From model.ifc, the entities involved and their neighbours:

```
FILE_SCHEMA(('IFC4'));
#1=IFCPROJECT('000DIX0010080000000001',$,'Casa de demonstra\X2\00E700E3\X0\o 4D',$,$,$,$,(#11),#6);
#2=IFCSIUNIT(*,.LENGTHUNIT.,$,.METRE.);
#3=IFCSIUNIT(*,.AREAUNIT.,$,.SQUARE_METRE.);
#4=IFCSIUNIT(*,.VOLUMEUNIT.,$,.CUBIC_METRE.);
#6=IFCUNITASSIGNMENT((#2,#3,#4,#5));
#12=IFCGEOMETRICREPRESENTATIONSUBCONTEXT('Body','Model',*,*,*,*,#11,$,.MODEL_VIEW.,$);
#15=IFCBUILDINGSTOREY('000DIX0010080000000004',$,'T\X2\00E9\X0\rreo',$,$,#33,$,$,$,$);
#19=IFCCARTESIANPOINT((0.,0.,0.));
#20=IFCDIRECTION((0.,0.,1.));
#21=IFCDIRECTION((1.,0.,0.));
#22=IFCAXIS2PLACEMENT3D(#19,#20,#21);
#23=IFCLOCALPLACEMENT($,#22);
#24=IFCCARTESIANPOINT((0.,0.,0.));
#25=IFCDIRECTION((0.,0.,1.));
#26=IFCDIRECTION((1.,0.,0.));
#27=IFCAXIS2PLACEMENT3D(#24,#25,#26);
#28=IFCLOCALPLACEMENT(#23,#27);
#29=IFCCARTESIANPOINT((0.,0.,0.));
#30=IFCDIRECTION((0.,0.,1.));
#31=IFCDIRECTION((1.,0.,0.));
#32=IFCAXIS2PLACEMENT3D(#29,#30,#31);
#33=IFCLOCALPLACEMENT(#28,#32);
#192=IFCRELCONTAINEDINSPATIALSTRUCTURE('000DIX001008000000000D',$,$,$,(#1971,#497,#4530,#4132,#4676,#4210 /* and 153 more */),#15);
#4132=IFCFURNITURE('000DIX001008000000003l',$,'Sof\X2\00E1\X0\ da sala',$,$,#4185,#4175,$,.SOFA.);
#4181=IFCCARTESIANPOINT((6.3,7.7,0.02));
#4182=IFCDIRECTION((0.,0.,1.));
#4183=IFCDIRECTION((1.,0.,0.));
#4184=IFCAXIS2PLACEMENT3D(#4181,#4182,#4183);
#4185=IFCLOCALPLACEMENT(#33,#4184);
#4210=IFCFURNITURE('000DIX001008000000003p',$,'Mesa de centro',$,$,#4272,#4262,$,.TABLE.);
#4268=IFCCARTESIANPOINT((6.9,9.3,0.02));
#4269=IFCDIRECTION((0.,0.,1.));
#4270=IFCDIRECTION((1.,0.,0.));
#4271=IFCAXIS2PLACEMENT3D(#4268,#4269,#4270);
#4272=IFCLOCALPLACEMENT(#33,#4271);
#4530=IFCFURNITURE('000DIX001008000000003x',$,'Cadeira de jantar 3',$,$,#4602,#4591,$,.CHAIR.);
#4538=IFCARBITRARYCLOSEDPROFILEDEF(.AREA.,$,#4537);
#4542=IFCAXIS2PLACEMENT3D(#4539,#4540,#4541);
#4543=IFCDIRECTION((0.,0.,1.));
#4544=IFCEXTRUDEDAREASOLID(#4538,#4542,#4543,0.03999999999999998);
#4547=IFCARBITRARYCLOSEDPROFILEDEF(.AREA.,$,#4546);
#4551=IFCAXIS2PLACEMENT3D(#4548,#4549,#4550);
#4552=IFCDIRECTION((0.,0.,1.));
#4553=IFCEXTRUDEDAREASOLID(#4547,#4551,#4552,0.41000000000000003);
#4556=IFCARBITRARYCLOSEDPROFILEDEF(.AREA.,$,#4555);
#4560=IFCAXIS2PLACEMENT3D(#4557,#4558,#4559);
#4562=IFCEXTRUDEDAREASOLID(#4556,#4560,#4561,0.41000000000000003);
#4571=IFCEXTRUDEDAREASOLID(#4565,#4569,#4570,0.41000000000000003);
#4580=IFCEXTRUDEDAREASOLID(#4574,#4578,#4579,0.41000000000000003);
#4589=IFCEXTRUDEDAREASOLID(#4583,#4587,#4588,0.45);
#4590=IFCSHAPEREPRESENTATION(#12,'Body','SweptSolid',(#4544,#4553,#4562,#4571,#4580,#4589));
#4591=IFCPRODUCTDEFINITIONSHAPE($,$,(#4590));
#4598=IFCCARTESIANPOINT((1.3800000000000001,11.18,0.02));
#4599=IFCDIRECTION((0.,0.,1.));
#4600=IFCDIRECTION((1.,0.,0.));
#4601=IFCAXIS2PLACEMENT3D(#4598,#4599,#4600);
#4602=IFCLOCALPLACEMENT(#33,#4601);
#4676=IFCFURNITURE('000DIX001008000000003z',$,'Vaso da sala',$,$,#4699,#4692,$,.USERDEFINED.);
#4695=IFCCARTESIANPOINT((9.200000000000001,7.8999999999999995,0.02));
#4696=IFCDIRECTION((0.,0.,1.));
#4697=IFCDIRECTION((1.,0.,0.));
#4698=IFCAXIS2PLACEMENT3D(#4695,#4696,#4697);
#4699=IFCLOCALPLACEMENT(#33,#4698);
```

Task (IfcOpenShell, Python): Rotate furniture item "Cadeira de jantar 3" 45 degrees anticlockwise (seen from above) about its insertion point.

```python
import ifcopenshell
import ifcopenshell.api.geometry
import ifcopenshell.util.placement

model = ifcopenshell.open("model.ifc")

item = model.by_guid("000DIX001008000000003x")
matrix = ifcopenshell.util.placement.get_local_placement(item.ObjectPlacement)
matrix = matrix @ ifcopenshell.util.placement.rotation(45, "Z")
ifcopenshell.api.geometry.edit_object_placement(model, product=item, matrix=matrix, is_si=False)

print(ifcopenshell.util.placement.get_local_placement(item.ObjectPlacement).round(3) + 0.0)

model.write("model_v2.ifc")
```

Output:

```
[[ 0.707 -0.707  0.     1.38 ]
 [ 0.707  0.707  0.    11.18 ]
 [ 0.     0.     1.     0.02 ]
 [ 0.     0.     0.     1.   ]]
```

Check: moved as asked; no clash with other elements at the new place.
